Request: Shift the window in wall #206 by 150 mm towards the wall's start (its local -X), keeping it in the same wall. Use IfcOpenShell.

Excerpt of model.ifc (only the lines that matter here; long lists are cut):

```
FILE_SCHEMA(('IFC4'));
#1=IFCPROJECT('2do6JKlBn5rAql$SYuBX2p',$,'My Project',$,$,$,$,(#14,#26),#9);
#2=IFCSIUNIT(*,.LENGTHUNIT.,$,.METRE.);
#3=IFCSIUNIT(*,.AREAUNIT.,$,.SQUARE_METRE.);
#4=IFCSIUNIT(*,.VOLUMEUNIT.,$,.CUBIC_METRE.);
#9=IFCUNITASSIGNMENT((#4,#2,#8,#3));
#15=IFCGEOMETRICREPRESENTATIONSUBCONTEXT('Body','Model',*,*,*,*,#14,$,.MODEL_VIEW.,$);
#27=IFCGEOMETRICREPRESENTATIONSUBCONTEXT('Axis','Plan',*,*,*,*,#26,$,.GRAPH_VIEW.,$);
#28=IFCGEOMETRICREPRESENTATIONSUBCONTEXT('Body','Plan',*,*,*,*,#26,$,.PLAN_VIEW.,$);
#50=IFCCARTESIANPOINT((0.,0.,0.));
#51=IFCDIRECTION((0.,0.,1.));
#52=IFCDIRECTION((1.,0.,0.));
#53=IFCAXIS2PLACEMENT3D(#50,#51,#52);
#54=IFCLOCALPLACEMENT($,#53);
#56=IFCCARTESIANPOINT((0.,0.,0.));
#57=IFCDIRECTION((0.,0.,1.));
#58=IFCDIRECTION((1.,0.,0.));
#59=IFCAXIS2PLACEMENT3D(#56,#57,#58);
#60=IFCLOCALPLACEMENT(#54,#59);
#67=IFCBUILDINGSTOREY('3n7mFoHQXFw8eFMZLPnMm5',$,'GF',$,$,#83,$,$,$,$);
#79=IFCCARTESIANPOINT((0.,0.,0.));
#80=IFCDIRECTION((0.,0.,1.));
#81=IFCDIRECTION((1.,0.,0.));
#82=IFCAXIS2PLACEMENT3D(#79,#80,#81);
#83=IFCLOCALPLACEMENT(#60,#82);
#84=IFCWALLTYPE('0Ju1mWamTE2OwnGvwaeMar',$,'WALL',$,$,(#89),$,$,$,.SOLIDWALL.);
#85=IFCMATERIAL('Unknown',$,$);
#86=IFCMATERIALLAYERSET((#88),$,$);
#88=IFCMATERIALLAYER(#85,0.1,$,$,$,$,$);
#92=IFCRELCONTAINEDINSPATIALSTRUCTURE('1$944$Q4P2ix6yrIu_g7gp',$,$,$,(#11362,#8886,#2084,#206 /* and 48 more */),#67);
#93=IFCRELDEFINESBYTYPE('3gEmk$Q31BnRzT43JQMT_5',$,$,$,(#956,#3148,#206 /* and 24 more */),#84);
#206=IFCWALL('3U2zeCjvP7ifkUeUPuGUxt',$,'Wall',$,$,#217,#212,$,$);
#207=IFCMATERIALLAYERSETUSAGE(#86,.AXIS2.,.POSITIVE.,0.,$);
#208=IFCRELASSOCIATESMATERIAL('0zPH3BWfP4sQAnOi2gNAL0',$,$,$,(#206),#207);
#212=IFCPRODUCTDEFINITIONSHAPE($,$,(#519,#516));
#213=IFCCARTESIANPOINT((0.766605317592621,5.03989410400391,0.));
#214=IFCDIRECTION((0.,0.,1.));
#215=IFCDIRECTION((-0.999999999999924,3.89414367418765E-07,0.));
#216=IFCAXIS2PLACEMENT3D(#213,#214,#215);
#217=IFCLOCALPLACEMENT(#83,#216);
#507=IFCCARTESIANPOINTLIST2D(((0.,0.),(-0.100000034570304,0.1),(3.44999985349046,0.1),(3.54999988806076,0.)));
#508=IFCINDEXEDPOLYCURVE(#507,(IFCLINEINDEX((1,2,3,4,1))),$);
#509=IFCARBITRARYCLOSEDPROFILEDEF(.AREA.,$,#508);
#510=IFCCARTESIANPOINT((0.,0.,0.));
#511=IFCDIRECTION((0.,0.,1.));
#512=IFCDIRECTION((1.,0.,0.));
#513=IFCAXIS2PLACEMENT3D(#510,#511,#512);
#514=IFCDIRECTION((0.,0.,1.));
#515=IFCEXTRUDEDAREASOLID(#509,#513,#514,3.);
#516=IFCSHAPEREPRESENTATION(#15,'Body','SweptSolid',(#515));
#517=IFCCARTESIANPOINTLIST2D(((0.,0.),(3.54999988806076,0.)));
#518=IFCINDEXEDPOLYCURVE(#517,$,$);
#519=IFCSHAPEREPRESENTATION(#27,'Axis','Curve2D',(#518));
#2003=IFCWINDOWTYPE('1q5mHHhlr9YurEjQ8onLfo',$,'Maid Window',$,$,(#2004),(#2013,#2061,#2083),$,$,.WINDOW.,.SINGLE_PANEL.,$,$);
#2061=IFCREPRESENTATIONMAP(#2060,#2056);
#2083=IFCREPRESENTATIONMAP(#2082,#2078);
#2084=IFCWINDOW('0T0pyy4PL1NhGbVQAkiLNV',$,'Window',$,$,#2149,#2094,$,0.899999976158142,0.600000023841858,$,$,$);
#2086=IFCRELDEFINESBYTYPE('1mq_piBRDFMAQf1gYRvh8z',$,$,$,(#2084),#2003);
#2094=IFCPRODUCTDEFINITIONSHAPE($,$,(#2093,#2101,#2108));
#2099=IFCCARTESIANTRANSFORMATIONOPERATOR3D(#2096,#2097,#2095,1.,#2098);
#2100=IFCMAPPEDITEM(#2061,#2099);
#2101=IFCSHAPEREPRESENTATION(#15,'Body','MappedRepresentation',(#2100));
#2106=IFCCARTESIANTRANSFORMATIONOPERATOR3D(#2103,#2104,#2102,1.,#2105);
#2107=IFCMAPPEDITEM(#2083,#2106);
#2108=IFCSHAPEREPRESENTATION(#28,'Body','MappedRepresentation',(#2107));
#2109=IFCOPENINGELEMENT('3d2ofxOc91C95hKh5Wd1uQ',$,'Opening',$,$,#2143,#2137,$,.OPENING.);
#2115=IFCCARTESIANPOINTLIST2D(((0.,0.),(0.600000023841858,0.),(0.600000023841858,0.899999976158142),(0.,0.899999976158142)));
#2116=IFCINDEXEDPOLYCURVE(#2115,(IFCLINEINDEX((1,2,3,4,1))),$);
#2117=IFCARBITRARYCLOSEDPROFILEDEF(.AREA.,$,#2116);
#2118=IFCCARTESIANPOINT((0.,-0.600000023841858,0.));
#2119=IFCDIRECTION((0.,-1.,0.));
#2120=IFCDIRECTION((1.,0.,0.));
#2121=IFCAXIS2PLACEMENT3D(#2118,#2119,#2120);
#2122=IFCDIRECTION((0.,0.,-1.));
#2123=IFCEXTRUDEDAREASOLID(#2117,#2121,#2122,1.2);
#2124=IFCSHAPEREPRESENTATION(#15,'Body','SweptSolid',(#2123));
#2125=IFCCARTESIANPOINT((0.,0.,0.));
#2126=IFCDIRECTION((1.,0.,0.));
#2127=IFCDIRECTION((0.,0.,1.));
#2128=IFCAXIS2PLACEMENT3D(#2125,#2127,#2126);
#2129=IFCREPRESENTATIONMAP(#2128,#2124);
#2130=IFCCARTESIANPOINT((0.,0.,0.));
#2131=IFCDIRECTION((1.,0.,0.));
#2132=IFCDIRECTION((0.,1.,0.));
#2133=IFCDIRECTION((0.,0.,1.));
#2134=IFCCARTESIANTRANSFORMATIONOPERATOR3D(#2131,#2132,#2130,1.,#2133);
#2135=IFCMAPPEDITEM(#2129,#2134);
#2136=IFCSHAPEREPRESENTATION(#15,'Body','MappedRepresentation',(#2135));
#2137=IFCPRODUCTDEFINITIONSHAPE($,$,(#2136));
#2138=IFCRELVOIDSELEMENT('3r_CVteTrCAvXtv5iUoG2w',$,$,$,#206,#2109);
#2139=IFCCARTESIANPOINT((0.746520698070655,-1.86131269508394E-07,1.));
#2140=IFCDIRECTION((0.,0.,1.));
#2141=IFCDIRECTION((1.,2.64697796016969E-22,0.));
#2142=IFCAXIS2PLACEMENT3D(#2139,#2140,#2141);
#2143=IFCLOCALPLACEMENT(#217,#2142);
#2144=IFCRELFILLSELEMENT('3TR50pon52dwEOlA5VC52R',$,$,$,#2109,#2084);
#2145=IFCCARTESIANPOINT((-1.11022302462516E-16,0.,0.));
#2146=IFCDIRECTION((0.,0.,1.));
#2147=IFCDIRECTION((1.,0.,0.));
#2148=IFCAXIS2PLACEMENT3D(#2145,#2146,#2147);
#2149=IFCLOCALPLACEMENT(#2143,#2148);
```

```python
import ifcopenshell
import ifcopenshell.api.geometry
import ifcopenshell.util.placement

model = ifcopenshell.open("model.ifc")

window = model.by_guid("0T0pyy4PL1NhGbVQAkiLNV")
opening = window.FillsVoids[0].RelatingOpeningElement
wall = opening.VoidsElements[0].RelatingBuildingElement

wall_matrix = ifcopenshell.util.placement.get_local_placement(wall.ObjectPlacement)
shift = wall_matrix[:3, 0] * -0.15
before = ifcopenshell.util.placement.get_local_placement(window.ObjectPlacement)[:3, 3].copy()

# The window is placed relative to its opening, so it follows when the opening moves.
matrix = ifcopenshell.util.placement.get_local_placement(opening.ObjectPlacement)
matrix[:3, 3] += shift
ifcopenshell.api.geometry.edit_object_placement(
    model, product=opening, matrix=matrix, is_si=False, should_transform_children=True
)

after = ifcopenshell.util.placement.get_local_placement(window.ObjectPlacement)[:3, 3]
print("window moved by", (after - before).round(3) + 0.0)

model.write("model_v2.ifc")
```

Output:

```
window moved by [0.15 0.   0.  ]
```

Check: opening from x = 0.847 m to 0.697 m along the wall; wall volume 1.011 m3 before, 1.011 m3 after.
